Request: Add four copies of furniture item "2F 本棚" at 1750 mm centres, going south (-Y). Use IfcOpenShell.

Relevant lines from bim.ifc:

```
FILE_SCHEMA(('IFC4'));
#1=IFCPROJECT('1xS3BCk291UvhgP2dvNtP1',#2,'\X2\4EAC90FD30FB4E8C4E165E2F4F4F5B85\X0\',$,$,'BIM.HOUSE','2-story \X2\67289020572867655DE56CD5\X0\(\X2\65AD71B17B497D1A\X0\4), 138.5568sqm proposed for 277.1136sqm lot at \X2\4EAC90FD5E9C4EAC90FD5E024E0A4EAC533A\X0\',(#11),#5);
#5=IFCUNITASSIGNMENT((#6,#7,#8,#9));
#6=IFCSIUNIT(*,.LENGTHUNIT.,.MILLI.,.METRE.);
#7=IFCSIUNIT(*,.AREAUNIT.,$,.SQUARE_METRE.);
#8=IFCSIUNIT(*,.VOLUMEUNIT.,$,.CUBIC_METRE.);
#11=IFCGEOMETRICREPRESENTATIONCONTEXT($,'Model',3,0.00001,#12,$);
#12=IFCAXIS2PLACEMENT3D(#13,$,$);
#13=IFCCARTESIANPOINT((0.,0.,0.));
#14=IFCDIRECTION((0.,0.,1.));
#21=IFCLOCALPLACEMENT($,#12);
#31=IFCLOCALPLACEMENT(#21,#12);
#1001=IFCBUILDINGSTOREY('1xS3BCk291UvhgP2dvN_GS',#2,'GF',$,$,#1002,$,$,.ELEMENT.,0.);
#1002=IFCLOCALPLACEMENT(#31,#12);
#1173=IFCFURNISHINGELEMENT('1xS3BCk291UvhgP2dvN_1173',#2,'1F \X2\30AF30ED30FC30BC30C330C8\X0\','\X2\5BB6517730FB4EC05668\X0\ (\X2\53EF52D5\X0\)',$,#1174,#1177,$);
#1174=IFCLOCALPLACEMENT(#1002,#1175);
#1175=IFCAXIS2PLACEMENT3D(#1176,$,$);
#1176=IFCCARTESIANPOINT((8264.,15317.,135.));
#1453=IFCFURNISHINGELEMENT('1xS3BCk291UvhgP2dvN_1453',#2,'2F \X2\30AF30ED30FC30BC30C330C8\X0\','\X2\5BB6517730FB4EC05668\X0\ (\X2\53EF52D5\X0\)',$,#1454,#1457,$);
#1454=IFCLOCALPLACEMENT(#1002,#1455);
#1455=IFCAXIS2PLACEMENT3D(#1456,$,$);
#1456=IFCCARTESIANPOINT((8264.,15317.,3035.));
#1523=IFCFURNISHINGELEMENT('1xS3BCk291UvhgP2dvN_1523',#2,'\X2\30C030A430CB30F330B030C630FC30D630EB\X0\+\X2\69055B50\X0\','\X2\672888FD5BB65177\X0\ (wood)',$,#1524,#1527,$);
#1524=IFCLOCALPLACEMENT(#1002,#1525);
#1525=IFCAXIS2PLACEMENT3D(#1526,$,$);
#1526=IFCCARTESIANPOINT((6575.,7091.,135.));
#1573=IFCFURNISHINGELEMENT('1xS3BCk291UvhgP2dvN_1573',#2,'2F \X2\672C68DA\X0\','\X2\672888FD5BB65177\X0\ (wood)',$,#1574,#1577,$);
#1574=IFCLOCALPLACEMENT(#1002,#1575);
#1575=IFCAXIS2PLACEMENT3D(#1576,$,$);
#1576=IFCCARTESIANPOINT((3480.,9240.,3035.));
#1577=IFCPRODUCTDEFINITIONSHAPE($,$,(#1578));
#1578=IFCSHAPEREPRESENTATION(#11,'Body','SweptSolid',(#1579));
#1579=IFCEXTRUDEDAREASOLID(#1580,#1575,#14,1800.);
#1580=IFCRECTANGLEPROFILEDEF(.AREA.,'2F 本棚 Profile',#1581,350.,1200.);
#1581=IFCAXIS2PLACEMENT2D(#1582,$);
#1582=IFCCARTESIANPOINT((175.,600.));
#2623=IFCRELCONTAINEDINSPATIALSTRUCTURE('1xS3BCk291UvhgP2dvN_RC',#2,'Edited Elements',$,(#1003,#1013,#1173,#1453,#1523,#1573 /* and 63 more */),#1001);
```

```python
import numpy as np
import ifcopenshell
import ifcopenshell.api.geometry
import ifcopenshell.api.root
import ifcopenshell.util.element
import ifcopenshell.util.placement

model = ifcopenshell.open("bim.ifc")


def reuse_history(source, copy):
    """copy_class also copies each property set's owner history, people and application; keep the originals."""
    for rel in copy.IsDefinedBy:
        if rel.is_a("IfcRelDefinesByProperties") and (history := rel.RelatingPropertyDefinition.OwnerHistory):
            rel.RelatingPropertyDefinition.OwnerHistory = source.OwnerHistory
            ifcopenshell.util.element.remove_deep2(model, history)


source = model.by_guid("1xS3BCk291UvhgP2dvN_1573")
base = ifcopenshell.util.placement.get_local_placement(source.ObjectPlacement)
step = np.array([0.0, -1.0, 0.0]) * 1750.0

for i in range(1, 5):
    copy = ifcopenshell.api.root.copy_class(model, product=source)
    copy.Representation = ifcopenshell.util.element.copy_deep(
        model, source.Representation, exclude=["IfcGeometricRepresentationContext", "IfcRepresentationMap"]
    )
    reuse_history(source, copy)
    matrix = base.copy()
    matrix[:3, 3] += i * step
    print("added at", matrix[:3, 3].round(3) + 0.0)
    ifcopenshell.api.geometry.edit_object_placement(model, product=copy, matrix=matrix, is_si=False)

model.write("bim_updated.ifc")
```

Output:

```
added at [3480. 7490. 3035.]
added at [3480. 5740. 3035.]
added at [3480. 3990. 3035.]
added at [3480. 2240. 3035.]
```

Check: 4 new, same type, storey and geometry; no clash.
